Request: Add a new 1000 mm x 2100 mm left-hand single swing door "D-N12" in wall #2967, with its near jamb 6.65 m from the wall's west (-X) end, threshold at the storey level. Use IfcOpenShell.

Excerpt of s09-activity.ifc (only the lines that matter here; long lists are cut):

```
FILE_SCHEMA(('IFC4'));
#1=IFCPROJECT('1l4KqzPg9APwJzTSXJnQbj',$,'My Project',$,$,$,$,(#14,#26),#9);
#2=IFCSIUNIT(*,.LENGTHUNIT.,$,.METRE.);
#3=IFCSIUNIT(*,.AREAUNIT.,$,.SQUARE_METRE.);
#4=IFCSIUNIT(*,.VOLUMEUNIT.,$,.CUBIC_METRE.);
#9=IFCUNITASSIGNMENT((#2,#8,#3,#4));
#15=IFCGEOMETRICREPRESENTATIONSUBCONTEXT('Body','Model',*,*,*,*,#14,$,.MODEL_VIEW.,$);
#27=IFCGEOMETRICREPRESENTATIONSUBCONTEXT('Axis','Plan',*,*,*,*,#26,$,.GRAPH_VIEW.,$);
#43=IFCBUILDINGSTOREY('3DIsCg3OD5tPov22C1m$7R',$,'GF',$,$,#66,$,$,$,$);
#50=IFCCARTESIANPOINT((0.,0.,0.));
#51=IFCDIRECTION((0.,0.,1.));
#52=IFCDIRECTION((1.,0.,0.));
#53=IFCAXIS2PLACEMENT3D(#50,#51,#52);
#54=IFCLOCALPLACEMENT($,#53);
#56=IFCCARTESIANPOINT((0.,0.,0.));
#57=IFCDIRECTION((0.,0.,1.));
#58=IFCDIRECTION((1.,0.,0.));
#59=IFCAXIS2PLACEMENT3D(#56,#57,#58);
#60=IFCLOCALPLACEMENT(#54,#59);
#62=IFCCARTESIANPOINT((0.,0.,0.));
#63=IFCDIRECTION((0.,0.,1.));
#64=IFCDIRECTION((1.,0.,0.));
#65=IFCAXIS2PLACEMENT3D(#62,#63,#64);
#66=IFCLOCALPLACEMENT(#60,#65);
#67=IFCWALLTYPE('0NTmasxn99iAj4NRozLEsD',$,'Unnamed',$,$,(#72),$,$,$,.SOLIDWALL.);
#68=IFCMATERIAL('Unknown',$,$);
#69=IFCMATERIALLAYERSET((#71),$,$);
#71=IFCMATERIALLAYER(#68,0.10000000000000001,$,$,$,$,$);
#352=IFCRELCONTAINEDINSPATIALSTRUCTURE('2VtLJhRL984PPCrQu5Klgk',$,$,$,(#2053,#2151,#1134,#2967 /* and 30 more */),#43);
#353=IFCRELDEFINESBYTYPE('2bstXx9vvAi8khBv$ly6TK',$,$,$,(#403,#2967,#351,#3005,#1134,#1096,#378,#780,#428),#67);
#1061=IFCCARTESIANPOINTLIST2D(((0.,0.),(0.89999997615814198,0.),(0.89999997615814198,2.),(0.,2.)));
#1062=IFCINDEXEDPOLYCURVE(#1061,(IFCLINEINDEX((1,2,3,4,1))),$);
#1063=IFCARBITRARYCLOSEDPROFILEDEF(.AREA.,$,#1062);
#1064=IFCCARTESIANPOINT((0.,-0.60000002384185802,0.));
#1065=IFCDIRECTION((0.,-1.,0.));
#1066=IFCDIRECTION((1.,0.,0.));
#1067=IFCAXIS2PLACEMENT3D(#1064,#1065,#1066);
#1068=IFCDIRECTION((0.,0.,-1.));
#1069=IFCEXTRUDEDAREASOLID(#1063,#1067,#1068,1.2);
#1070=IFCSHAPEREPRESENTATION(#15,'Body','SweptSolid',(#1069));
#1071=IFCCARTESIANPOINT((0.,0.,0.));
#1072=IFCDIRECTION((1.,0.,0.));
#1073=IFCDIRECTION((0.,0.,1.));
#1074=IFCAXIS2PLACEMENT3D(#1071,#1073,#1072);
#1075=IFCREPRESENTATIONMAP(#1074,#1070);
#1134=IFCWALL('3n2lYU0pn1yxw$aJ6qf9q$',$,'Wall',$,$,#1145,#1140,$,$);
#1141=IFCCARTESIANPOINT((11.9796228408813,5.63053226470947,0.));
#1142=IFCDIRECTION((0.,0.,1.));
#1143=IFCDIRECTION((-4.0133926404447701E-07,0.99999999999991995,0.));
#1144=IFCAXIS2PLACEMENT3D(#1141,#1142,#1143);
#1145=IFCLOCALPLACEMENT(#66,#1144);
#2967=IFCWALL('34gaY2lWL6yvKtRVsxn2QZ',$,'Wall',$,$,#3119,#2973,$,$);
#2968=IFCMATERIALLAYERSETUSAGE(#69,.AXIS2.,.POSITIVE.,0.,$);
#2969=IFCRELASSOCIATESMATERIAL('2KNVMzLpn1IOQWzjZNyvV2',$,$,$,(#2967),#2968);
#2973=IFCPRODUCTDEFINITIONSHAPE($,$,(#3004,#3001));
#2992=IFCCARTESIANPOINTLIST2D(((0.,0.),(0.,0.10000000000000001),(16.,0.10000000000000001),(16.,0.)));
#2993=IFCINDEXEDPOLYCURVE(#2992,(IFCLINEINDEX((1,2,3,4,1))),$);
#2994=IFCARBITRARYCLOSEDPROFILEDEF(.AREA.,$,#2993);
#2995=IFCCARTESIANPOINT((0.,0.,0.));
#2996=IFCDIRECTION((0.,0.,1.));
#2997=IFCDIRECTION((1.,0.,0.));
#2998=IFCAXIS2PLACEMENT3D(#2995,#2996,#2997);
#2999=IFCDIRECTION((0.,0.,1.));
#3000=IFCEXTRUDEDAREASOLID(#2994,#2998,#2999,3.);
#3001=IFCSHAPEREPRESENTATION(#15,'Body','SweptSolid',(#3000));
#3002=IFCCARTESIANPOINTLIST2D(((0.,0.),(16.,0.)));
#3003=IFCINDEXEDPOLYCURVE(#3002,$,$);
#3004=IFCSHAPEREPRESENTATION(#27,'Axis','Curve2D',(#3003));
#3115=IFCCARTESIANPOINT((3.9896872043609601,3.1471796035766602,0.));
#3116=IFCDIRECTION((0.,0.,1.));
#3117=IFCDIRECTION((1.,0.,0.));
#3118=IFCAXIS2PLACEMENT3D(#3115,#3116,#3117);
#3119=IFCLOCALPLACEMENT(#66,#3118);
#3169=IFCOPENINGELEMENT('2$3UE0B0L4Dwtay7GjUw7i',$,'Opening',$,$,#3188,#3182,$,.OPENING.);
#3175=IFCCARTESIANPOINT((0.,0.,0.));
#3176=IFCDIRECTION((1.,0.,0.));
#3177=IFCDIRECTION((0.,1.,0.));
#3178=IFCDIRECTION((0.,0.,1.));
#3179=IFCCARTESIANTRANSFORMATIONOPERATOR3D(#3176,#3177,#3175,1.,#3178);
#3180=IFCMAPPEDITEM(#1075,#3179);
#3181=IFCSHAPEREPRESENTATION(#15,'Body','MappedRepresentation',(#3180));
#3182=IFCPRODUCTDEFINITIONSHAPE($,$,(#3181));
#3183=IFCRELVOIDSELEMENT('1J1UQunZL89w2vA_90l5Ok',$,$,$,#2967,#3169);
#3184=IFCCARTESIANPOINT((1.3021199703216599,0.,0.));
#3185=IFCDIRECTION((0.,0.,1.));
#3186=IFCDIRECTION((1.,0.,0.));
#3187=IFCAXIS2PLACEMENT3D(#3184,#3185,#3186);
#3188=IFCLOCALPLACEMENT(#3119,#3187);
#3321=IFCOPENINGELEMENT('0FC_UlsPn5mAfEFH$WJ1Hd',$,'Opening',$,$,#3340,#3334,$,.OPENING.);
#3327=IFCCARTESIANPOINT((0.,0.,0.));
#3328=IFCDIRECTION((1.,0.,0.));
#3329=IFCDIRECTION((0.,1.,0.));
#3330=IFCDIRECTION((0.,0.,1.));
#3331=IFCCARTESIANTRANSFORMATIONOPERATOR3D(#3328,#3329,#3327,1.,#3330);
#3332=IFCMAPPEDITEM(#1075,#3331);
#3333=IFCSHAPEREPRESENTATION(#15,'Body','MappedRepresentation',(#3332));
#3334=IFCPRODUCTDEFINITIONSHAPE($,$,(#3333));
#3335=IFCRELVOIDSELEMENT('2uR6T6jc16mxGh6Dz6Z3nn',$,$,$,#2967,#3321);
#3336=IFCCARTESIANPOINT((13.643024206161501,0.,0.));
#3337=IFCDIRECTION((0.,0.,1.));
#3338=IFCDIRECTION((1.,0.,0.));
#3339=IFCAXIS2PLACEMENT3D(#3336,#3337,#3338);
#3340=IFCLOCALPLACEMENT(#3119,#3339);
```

```python
import numpy as np
import ifcopenshell
import ifcopenshell.api.feature
import ifcopenshell.api.geometry
import ifcopenshell.api.root
import ifcopenshell.api.spatial
import ifcopenshell.geom
import ifcopenshell.util.element
import ifcopenshell.util.placement
import ifcopenshell.util.representation
import ifcopenshell.util.shape
import ifcopenshell.util.unit

model = ifcopenshell.open("s09-activity.ifc")
unit_scale = ifcopenshell.util.unit.calculate_unit_scale(model)
settings = ifcopenshell.geom.settings()


def volume(element):
    """Net volume in cubic metres, openings subtracted."""
    shape = ifcopenshell.geom.create_shape(settings, element)
    return ifcopenshell.util.shape.get_volume(shape.geometry)


wall = model.by_guid("34gaY2lWL6yvKtRVsxn2QZ")
storey = ifcopenshell.util.element.get_container(wall, ifc_class="IfcBuildingStorey")
context = ifcopenshell.util.representation.get_context(model, "Model", "Body", "MODEL_VIEW")
before = volume(wall)

width, height, from_end, sill = 1, 2.1, 6.65, 0.0  # metres

# The wall runs along its own X axis, and the end named is its -X end.
wall_shape = ifcopenshell.geom.create_shape(settings, wall)
x, y, z = ifcopenshell.util.shape.get_vertices(wall_shape.geometry).T
start = x.min() + from_end
face, thickness = float(y.min()), float(y.max() - y.min())
wall_matrix = ifcopenshell.util.placement.get_local_placement(wall.ObjectPlacement)
level = ifcopenshell.util.placement.get_local_placement(storey.ObjectPlacement)[2, 3]


def in_wall(x, y):
    """Placement at x, y metres in the wall's axes, at sill height."""
    matrix = wall_matrix.copy()
    matrix[:, 3] = wall_matrix @ np.array([x / unit_scale, y / unit_scale, 0.0, 1.0])
    matrix[2, 3] = level + sill / unit_scale
    return matrix


# Opening: a box that overshoots both wall faces by 50 mm.
opening = ifcopenshell.api.root.create_entity(model, ifc_class="IfcOpeningElement", predefined_type="OPENING")
box = ifcopenshell.api.geometry.add_wall_representation(
    model, context=context, length=width, height=height, thickness=thickness + 0.1
)
ifcopenshell.api.geometry.assign_representation(model, product=opening, representation=box)
ifcopenshell.api.geometry.edit_object_placement(model, product=opening, matrix=in_wall(start, face - 0.05), is_si=False)
ifcopenshell.api.feature.add_feature(model, feature=opening, element=wall)

door = ifcopenshell.api.root.create_entity(model, ifc_class="IfcDoor", name="D-N12", predefined_type="DOOR")
door.OverallWidth, door.OverallHeight = width / unit_scale, height / unit_scale
door.OperationType = "SINGLE_SWING_LEFT"
body = ifcopenshell.api.geometry.add_door_representation(
    model,
    context=context,
    overall_width=door.OverallWidth,
    overall_height=door.OverallHeight,
    operation_type="SINGLE_SWING_LEFT",
    lining_properties={"LiningDepth": thickness / unit_scale, "ThresholdDepth": thickness / unit_scale},
)
ifcopenshell.api.geometry.assign_representation(model, product=door, representation=body)
ifcopenshell.api.spatial.assign_container(model, products=[door], relating_structure=storey)
ifcopenshell.api.feature.add_filling(model, opening=opening, element=door)

# The lining spans the wall, so the door starts at the wall face.
ifcopenshell.api.geometry.edit_object_placement(model, product=door, matrix=in_wall(start, face), is_si=False)

after = volume(wall)

print(f"wall volume {before:.3f} -> {after:.3f} m3")

model.write("s09-activity-out.ifc")
```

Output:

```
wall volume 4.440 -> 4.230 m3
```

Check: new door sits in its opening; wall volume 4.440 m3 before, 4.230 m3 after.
